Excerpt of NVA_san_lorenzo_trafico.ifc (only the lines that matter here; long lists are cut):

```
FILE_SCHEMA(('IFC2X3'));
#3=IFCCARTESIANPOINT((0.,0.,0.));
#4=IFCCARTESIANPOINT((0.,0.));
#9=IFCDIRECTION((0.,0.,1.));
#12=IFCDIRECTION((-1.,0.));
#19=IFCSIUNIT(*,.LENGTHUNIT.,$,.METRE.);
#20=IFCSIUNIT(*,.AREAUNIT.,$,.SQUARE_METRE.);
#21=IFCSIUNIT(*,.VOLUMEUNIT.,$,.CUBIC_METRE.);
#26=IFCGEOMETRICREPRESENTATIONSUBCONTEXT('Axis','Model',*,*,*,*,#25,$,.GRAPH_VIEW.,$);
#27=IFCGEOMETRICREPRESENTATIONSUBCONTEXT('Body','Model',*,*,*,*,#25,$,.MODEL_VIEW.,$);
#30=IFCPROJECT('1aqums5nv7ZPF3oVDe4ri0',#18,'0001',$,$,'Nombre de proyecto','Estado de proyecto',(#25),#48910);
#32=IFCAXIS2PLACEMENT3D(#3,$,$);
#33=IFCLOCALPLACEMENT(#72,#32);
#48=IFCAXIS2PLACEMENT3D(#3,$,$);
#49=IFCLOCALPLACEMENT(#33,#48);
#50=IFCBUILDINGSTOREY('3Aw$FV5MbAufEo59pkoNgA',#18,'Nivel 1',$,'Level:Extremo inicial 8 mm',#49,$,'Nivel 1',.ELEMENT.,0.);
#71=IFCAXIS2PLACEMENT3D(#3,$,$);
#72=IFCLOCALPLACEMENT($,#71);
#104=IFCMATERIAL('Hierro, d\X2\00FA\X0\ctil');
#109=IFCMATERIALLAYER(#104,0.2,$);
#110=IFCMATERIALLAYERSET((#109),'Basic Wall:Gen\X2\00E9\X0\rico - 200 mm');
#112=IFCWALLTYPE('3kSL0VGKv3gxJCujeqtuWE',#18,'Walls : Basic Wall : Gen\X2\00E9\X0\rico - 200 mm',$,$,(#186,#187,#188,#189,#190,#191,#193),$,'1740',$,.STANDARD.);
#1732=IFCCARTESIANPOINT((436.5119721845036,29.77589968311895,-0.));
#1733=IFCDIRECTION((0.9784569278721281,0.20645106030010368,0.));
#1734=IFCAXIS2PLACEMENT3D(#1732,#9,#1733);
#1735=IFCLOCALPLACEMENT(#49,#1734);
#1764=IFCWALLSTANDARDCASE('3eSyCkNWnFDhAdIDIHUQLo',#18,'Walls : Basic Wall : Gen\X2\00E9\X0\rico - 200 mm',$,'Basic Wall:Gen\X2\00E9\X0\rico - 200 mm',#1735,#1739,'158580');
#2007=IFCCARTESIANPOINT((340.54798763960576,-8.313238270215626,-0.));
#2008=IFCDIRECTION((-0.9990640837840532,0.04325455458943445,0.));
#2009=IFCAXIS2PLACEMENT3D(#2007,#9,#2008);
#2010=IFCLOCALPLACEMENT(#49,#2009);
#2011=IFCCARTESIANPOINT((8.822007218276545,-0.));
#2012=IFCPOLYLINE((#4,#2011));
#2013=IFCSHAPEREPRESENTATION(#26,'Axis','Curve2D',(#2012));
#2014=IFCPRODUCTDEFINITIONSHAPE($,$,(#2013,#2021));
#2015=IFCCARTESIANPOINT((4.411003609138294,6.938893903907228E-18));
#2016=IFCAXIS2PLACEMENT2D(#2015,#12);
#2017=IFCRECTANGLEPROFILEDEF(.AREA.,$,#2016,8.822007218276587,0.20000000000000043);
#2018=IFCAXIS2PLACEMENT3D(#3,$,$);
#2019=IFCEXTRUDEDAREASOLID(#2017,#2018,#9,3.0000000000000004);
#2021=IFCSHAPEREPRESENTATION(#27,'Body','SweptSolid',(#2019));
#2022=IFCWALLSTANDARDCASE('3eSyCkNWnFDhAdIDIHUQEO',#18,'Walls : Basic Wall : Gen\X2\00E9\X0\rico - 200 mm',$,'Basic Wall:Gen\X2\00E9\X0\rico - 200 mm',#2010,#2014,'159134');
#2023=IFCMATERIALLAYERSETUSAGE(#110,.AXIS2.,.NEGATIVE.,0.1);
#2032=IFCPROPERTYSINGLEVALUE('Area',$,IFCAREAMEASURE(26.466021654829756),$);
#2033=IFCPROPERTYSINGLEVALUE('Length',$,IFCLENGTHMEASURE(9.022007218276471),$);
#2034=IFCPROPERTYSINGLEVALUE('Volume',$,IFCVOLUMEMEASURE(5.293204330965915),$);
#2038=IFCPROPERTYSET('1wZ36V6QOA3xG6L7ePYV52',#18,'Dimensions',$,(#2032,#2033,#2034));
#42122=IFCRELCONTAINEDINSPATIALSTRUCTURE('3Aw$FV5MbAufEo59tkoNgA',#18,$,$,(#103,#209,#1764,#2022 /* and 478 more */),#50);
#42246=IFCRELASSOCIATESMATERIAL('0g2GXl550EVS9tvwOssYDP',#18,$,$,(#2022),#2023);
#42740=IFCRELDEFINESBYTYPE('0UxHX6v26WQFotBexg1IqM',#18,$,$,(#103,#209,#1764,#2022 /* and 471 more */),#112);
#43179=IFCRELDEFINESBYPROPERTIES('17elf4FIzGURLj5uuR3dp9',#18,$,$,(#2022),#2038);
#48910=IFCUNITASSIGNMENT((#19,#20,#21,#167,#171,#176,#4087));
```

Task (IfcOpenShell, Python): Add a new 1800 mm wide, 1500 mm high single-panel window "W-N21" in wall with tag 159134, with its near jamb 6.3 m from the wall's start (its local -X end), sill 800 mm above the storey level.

```python
import numpy as np
import ifcopenshell
import ifcopenshell.api.feature
import ifcopenshell.api.geometry
import ifcopenshell.api.pset
import ifcopenshell.api.root
import ifcopenshell.api.spatial
import ifcopenshell.api.type
import ifcopenshell.geom
import ifcopenshell.util.element
import ifcopenshell.util.placement
import ifcopenshell.util.representation
import ifcopenshell.util.shape
import ifcopenshell.util.unit

model = ifcopenshell.open("NVA_san_lorenzo_trafico.ifc")
unit_scale = ifcopenshell.util.unit.calculate_unit_scale(model)
area_scale = ifcopenshell.util.unit.calculate_unit_scale(model, "AREAUNIT")
volume_scale = ifcopenshell.util.unit.calculate_unit_scale(model, "VOLUMEUNIT")
settings = ifcopenshell.geom.settings()


def volume(element):
    """Net volume in cubic metres, openings subtracted."""
    shape = ifcopenshell.geom.create_shape(settings, element)
    return ifcopenshell.util.shape.get_volume(shape.geometry)


wall = model.by_guid("3eSyCkNWnFDhAdIDIHUQEO")
storey = ifcopenshell.util.element.get_container(wall, ifc_class="IfcBuildingStorey")
context = ifcopenshell.util.representation.get_context(model, "Model", "Body", "MODEL_VIEW")
before = volume(wall)

width, height, from_end, sill = 1.8, 1.5, 6.3, 0.8  # metres

# The wall runs along its own X axis, and the end named is its -X end.
wall_shape = ifcopenshell.geom.create_shape(settings, wall)
x, y, z = ifcopenshell.util.shape.get_vertices(wall_shape.geometry).T
start = x.min() + from_end
face, thickness = float(y.min()), float(y.max() - y.min())
wall_matrix = ifcopenshell.util.placement.get_local_placement(wall.ObjectPlacement)
level = ifcopenshell.util.placement.get_local_placement(storey.ObjectPlacement)[2, 3]


def in_wall(x, y):
    """Placement at x, y metres in the wall's axes, at sill height."""
    matrix = wall_matrix.copy()
    matrix[:, 3] = wall_matrix @ np.array([x / unit_scale, y / unit_scale, 0.0, 1.0])
    matrix[2, 3] = level + sill / unit_scale
    return matrix


# Opening: a box that overshoots both wall faces by 50 mm.
opening = ifcopenshell.api.root.create_entity(model, ifc_class="IfcOpeningElement")
box = ifcopenshell.api.geometry.add_wall_representation(
    model, context=context, length=width, height=height, thickness=thickness + 0.1
)
ifcopenshell.api.geometry.assign_representation(model, product=opening, representation=box)
ifcopenshell.api.geometry.edit_object_placement(model, product=opening, matrix=in_wall(start, face - 0.05), is_si=False)
ifcopenshell.api.feature.add_feature(model, feature=opening, element=wall)

window = ifcopenshell.api.root.create_entity(model, ifc_class="IfcWindow", name="W-N21")
window.OverallWidth, window.OverallHeight = width / unit_scale, height / unit_scale
body = ifcopenshell.api.geometry.add_window_representation(
    model,
    context=context,
    overall_width=window.OverallWidth,
    overall_height=window.OverallHeight,
    partition_type="SINGLE_PANEL",
)
ifcopenshell.api.geometry.assign_representation(model, product=window, representation=body)
ifcopenshell.api.spatial.assign_container(model, products=[window], relating_structure=storey)
fills = ifcopenshell.api.feature.add_filling(model, opening=opening, element=window)
fills.OwnerHistory = window.OwnerHistory  # required in IFC2X3

# IFC2X3 keeps the operation on the window style.
style = ifcopenshell.api.root.create_entity(model, ifc_class="IfcWindowStyle", name="W-N21")
style.OperationType, style.ConstructionType = "SINGLE_PANEL", "NOTDEFINED"
style.ParameterTakesPrecedence = style.Sizeable = False
ifcopenshell.api.type.assign_type(model, related_objects=[window], relating_type=style)

# Centre the window in the wall's thickness.
ifcopenshell.api.geometry.edit_object_placement(model, product=window, matrix=in_wall(start, face), is_si=False)
window_shape = ifcopenshell.geom.create_shape(settings, window)
depth = ifcopenshell.util.shape.get_vertices(window_shape.geometry)[:, 1]
offset = face + thickness / 2 - (depth.min() + depth.max()) / 2
ifcopenshell.api.geometry.edit_object_placement(model, product=window, matrix=in_wall(start, offset), is_si=False)

after = volume(wall)

# Update the wall's stored quantities.
pset = model.by_id(ifcopenshell.util.element.get_pset(wall, "Dimensions", should_inherit=False)["id"])
ifcopenshell.api.pset.edit_pset(model, pset=pset, properties={
    "Area": model.create_entity("IfcAreaMeasure", after / thickness / area_scale),
    "Volume": model.create_entity("IfcVolumeMeasure", after / volume_scale),
})

print(f"wall volume {before:.3f} -> {after:.3f} m3")

model.write("NVA_san_lorenzo_trafico_rev.ifc")
```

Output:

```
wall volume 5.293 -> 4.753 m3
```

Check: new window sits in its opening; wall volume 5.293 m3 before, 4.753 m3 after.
